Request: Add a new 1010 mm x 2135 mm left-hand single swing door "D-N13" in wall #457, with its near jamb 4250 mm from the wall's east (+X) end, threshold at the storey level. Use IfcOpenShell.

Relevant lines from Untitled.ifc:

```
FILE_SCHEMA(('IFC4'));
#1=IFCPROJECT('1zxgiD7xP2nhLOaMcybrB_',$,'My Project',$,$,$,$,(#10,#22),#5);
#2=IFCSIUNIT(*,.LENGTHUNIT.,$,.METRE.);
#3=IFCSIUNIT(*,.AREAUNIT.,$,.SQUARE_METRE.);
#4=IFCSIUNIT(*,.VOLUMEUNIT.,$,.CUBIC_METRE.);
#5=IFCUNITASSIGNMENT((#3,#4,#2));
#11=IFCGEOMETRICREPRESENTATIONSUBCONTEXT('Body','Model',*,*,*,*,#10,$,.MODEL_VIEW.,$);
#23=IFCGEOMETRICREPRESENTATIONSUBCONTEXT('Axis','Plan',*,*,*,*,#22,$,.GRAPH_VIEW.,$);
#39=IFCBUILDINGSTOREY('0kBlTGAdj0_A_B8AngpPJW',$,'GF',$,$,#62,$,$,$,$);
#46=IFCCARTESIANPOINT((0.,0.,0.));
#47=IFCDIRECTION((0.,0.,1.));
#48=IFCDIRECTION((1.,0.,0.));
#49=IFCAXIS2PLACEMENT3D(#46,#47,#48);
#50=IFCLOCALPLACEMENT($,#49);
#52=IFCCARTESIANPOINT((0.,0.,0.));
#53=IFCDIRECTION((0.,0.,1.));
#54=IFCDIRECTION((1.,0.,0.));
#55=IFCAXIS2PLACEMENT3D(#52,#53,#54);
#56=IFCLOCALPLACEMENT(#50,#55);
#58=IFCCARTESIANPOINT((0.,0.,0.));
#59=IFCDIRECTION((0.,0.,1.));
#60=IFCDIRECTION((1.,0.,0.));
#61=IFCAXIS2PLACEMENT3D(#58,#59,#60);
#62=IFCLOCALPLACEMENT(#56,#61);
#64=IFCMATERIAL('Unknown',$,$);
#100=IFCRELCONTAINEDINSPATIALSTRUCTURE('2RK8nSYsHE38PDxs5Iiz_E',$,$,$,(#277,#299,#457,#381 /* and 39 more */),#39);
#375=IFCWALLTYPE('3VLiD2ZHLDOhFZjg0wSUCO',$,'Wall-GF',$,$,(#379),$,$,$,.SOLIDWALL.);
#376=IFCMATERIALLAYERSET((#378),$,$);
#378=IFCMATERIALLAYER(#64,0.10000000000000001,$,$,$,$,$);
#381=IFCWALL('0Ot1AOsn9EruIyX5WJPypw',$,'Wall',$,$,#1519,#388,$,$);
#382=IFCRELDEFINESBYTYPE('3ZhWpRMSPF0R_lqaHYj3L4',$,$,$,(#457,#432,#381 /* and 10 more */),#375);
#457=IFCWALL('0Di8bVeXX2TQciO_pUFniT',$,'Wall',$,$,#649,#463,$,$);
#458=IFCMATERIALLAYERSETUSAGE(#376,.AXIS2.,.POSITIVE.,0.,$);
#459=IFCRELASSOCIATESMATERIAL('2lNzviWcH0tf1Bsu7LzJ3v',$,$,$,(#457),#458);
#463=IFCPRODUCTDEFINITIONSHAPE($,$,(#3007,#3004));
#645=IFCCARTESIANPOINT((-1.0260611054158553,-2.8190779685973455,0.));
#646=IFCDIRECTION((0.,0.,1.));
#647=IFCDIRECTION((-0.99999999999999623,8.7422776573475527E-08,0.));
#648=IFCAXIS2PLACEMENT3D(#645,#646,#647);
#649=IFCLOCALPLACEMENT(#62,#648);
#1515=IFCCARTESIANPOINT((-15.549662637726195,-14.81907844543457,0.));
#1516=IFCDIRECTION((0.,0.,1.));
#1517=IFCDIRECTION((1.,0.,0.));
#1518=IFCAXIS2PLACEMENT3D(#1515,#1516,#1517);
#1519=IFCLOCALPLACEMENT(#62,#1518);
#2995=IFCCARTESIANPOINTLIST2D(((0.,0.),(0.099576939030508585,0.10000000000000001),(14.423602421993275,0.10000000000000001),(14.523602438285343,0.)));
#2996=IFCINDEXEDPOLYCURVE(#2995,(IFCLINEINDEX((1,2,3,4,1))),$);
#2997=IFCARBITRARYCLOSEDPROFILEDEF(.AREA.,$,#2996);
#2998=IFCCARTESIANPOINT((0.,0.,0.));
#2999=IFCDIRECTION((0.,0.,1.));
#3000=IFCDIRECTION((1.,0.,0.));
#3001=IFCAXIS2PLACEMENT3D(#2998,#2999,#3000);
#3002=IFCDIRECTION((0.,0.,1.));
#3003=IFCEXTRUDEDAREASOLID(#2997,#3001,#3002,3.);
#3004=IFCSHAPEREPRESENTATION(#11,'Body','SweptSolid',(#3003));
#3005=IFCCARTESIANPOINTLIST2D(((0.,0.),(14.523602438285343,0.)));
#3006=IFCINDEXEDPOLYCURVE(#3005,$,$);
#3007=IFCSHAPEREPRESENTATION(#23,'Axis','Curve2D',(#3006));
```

```python
import numpy as np
import ifcopenshell
import ifcopenshell.api.feature
import ifcopenshell.api.geometry
import ifcopenshell.api.root
import ifcopenshell.api.spatial
import ifcopenshell.geom
import ifcopenshell.util.element
import ifcopenshell.util.placement
import ifcopenshell.util.representation
import ifcopenshell.util.shape
import ifcopenshell.util.unit

model = ifcopenshell.open("Untitled.ifc")
unit_scale = ifcopenshell.util.unit.calculate_unit_scale(model)
settings = ifcopenshell.geom.settings()


def volume(element):
    """Net volume in cubic metres, openings subtracted."""
    shape = ifcopenshell.geom.create_shape(settings, element)
    return ifcopenshell.util.shape.get_volume(shape.geometry)


wall = model.by_guid("0Di8bVeXX2TQciO_pUFniT")
storey = ifcopenshell.util.element.get_container(wall, ifc_class="IfcBuildingStorey")
context = ifcopenshell.util.representation.get_context(model, "Model", "Body", "MODEL_VIEW")
before = volume(wall)

width, height, from_end, sill = 1.01, 2.135, 4.25, 0.0  # metres

# The wall runs along its own X axis, and the end named is its -X end.
wall_shape = ifcopenshell.geom.create_shape(settings, wall)
x, y, z = ifcopenshell.util.shape.get_vertices(wall_shape.geometry).T
start = x.min() + from_end
face, thickness = float(y.min()), float(y.max() - y.min())
wall_matrix = ifcopenshell.util.placement.get_local_placement(wall.ObjectPlacement)
level = ifcopenshell.util.placement.get_local_placement(storey.ObjectPlacement)[2, 3]


def in_wall(x, y):
    """Placement at x, y metres in the wall's axes, at sill height."""
    matrix = wall_matrix.copy()
    matrix[:, 3] = wall_matrix @ np.array([x / unit_scale, y / unit_scale, 0.0, 1.0])
    matrix[2, 3] = level + sill / unit_scale
    return matrix


# Opening: a box that overshoots both wall faces by 50 mm.
opening = ifcopenshell.api.root.create_entity(model, ifc_class="IfcOpeningElement", predefined_type="OPENING")
box = ifcopenshell.api.geometry.add_wall_representation(
    model, context=context, length=width, height=height, thickness=thickness + 0.1
)
ifcopenshell.api.geometry.assign_representation(model, product=opening, representation=box)
ifcopenshell.api.geometry.edit_object_placement(model, product=opening, matrix=in_wall(start, face - 0.05), is_si=False)
ifcopenshell.api.feature.add_feature(model, feature=opening, element=wall)

door = ifcopenshell.api.root.create_entity(model, ifc_class="IfcDoor", name="D-N13", predefined_type="DOOR")
door.OverallWidth, door.OverallHeight = width / unit_scale, height / unit_scale
door.OperationType = "SINGLE_SWING_LEFT"
body = ifcopenshell.api.geometry.add_door_representation(
    model,
    context=context,
    overall_width=door.OverallWidth,
    overall_height=door.OverallHeight,
    operation_type="SINGLE_SWING_LEFT",
    lining_properties={"LiningDepth": thickness / unit_scale, "ThresholdDepth": thickness / unit_scale},
)
ifcopenshell.api.geometry.assign_representation(model, product=door, representation=body)
ifcopenshell.api.spatial.assign_container(model, products=[door], relating_structure=storey)
ifcopenshell.api.feature.add_filling(model, opening=opening, element=door)

# The lining spans the wall, so the door starts at the wall face.
ifcopenshell.api.geometry.edit_object_placement(model, product=door, matrix=in_wall(start, face), is_si=False)

after = volume(wall)

print(f"wall volume {before:.3f} -> {after:.3f} m3")

model.write("Untitled_edited.ifc")
```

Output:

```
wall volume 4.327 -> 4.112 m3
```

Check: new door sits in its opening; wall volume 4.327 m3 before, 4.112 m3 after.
